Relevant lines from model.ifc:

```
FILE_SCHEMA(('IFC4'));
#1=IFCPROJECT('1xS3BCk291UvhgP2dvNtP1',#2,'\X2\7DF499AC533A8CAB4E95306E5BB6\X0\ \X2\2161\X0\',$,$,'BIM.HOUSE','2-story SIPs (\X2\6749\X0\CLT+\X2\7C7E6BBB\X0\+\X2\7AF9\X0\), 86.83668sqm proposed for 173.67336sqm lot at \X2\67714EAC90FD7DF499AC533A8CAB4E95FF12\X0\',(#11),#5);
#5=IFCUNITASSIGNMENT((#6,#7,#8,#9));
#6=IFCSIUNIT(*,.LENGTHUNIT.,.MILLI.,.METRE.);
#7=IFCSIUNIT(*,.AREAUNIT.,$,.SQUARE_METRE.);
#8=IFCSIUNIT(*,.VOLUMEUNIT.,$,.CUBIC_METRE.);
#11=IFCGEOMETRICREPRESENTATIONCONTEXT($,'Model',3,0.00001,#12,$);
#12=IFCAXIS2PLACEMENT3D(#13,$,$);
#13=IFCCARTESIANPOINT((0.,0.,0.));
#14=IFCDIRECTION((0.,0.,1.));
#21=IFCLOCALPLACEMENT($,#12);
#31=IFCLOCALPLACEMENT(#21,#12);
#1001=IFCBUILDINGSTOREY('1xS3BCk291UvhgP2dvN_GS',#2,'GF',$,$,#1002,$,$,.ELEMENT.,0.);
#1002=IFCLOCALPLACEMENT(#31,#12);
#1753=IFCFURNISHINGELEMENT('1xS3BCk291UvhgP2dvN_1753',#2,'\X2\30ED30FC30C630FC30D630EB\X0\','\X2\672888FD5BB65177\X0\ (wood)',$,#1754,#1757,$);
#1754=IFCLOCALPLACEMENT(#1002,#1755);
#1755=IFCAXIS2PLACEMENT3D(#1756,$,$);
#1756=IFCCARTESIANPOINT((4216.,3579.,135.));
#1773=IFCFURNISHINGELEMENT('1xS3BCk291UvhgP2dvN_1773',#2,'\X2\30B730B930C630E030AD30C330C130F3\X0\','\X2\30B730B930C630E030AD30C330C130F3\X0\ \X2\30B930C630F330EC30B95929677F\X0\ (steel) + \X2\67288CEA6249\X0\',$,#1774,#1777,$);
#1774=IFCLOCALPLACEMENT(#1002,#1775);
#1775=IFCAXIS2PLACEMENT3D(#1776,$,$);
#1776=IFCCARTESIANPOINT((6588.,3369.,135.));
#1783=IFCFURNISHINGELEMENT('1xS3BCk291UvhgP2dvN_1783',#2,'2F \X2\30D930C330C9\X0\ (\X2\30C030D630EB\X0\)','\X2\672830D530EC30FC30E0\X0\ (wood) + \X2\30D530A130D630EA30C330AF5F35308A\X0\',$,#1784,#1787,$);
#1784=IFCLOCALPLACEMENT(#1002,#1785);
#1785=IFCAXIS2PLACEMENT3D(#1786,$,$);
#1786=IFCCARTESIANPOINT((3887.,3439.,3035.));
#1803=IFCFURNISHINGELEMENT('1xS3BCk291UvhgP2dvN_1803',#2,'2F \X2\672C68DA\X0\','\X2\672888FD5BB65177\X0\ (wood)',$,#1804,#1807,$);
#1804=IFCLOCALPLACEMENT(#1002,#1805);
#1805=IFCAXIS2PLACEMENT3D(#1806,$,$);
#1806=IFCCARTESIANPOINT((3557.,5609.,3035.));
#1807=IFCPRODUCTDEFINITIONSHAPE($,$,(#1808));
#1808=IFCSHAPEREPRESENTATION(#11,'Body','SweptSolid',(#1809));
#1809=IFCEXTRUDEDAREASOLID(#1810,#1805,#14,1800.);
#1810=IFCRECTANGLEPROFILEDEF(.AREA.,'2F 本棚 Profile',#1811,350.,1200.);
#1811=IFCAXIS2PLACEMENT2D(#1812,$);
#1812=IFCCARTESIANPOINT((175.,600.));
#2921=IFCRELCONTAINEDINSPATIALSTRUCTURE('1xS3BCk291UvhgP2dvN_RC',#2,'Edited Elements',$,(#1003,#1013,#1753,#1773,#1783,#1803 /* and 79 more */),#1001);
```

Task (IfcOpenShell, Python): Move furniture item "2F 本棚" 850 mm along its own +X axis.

```python
import ifcopenshell
import ifcopenshell.api.geometry
import ifcopenshell.util.placement
import ifcopenshell.util.unit

model = ifcopenshell.open("model.ifc")
unit_scale = ifcopenshell.util.unit.calculate_unit_scale(model)

item = model.by_id(1803)
matrix = ifcopenshell.util.placement.get_local_placement(item.ObjectPlacement)
matrix[:3, 3] += matrix[:3, 0] * 0.85 / unit_scale
ifcopenshell.api.geometry.edit_object_placement(model, product=item, matrix=matrix, is_si=False)

print(ifcopenshell.util.placement.get_local_placement(item.ObjectPlacement).round(3) + 0.0)

model.write("model_updated.ifc")
```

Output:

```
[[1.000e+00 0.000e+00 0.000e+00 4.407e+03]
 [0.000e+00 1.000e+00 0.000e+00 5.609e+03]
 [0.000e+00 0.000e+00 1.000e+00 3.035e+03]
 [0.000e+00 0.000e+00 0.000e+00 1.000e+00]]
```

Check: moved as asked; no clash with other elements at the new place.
